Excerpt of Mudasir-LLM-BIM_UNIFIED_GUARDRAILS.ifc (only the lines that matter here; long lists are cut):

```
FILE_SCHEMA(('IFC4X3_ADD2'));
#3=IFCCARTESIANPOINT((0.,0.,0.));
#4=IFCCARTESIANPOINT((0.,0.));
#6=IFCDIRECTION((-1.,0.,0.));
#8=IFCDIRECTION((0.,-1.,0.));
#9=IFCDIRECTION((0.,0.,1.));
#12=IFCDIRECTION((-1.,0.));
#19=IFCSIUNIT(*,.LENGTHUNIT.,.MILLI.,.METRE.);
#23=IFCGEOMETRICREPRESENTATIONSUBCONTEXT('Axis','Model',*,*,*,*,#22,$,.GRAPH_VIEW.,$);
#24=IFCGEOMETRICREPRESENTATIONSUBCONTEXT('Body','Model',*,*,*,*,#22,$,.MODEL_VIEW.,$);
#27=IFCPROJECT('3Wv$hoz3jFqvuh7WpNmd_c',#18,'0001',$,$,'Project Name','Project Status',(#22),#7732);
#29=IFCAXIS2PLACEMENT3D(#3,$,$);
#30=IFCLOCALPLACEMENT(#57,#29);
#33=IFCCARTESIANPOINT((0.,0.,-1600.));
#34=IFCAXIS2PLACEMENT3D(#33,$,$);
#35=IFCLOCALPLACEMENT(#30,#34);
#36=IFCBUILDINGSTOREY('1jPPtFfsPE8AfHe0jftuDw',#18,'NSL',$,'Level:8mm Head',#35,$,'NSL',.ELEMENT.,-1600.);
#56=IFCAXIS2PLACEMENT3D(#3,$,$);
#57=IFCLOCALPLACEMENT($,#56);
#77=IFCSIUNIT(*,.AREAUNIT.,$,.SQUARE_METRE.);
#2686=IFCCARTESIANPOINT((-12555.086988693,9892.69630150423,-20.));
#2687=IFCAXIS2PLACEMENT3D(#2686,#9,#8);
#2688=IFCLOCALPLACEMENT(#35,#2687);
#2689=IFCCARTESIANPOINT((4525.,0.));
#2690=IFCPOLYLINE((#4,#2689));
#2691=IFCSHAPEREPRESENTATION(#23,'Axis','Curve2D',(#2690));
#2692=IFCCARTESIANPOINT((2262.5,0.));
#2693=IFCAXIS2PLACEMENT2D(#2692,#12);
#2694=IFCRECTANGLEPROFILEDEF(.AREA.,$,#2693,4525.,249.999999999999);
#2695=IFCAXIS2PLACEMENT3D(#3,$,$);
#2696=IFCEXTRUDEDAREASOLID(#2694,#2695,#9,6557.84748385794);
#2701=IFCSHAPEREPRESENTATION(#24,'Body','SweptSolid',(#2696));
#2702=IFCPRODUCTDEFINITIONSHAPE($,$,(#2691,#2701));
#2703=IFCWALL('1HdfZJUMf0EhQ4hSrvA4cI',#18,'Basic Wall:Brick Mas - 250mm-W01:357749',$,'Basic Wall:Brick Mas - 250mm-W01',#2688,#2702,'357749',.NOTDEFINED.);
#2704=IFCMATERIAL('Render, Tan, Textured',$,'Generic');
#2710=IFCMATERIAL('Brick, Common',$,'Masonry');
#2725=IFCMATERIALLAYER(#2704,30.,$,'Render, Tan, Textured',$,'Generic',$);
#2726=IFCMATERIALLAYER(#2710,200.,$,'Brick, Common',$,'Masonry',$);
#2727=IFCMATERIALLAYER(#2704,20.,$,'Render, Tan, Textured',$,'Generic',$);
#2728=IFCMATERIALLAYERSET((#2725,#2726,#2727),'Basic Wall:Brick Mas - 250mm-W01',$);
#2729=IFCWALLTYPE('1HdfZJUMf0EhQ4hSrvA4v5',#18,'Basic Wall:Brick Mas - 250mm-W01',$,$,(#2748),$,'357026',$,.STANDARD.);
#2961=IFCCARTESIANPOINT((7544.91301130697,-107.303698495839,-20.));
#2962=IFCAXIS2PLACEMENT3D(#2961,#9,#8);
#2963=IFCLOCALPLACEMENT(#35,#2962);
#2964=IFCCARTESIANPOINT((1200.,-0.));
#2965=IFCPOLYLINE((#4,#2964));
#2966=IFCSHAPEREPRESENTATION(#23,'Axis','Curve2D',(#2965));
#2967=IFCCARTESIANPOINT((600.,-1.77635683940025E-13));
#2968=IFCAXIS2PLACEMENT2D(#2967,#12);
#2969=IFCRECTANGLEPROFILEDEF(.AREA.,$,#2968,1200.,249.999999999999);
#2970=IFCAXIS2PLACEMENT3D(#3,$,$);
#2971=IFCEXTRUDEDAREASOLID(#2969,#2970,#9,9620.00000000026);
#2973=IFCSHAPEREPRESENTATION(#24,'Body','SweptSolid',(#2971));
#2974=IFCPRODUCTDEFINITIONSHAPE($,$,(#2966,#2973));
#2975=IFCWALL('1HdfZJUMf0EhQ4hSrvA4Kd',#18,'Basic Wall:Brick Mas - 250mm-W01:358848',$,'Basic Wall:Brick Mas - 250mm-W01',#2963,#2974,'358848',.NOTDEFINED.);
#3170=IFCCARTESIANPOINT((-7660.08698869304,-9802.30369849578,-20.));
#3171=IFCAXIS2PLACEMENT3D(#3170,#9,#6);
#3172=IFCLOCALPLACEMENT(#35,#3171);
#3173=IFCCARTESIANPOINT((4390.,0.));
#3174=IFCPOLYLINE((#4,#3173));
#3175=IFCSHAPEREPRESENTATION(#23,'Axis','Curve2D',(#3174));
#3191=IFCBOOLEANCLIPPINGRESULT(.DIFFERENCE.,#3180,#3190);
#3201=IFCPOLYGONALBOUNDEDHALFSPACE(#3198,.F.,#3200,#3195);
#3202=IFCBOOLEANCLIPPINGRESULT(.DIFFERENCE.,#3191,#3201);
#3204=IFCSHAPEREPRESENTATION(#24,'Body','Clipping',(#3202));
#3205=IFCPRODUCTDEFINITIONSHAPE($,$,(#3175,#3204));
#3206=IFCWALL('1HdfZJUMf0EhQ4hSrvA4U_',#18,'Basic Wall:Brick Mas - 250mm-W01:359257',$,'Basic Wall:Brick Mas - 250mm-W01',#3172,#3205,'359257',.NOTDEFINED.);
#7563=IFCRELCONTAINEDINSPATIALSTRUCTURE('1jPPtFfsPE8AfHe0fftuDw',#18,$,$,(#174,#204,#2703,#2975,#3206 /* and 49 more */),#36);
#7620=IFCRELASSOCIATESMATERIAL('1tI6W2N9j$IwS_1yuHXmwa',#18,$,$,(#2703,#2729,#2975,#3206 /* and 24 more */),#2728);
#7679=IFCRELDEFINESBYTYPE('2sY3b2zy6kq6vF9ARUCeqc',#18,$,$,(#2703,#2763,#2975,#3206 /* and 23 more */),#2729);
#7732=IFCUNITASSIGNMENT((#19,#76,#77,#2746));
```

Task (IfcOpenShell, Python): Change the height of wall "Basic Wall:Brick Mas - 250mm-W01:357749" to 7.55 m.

```python
import ifcopenshell
import ifcopenshell.geom
import ifcopenshell.util.representation
import ifcopenshell.util.shape

model = ifcopenshell.open("Mudasir-LLM-BIM_UNIFIED_GUARDRAILS.ifc")
settings = ifcopenshell.geom.settings()


def volume(element):
    """Net volume in cubic metres, openings subtracted."""
    shape = ifcopenshell.geom.create_shape(settings, element)
    return ifcopenshell.util.shape.get_volume(shape.geometry)


wall = model.by_id(2703)
before = volume(wall)

body = ifcopenshell.util.representation.get_representation(wall, "Model", "Body")
solid = body.Items[0]
old_height = solid.Depth
solid.Depth = 7550.0
after = volume(wall)

print(f"height {old_height:g} -> {solid.Depth:g}, volume {before:.3f} -> {after:.3f} m3")

model.write("Mudasir-LLM-BIM_UNIFIED_GUARDRAILS_updated.ifc")
```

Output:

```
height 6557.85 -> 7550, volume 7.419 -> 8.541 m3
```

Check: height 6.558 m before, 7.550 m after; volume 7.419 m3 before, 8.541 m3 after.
